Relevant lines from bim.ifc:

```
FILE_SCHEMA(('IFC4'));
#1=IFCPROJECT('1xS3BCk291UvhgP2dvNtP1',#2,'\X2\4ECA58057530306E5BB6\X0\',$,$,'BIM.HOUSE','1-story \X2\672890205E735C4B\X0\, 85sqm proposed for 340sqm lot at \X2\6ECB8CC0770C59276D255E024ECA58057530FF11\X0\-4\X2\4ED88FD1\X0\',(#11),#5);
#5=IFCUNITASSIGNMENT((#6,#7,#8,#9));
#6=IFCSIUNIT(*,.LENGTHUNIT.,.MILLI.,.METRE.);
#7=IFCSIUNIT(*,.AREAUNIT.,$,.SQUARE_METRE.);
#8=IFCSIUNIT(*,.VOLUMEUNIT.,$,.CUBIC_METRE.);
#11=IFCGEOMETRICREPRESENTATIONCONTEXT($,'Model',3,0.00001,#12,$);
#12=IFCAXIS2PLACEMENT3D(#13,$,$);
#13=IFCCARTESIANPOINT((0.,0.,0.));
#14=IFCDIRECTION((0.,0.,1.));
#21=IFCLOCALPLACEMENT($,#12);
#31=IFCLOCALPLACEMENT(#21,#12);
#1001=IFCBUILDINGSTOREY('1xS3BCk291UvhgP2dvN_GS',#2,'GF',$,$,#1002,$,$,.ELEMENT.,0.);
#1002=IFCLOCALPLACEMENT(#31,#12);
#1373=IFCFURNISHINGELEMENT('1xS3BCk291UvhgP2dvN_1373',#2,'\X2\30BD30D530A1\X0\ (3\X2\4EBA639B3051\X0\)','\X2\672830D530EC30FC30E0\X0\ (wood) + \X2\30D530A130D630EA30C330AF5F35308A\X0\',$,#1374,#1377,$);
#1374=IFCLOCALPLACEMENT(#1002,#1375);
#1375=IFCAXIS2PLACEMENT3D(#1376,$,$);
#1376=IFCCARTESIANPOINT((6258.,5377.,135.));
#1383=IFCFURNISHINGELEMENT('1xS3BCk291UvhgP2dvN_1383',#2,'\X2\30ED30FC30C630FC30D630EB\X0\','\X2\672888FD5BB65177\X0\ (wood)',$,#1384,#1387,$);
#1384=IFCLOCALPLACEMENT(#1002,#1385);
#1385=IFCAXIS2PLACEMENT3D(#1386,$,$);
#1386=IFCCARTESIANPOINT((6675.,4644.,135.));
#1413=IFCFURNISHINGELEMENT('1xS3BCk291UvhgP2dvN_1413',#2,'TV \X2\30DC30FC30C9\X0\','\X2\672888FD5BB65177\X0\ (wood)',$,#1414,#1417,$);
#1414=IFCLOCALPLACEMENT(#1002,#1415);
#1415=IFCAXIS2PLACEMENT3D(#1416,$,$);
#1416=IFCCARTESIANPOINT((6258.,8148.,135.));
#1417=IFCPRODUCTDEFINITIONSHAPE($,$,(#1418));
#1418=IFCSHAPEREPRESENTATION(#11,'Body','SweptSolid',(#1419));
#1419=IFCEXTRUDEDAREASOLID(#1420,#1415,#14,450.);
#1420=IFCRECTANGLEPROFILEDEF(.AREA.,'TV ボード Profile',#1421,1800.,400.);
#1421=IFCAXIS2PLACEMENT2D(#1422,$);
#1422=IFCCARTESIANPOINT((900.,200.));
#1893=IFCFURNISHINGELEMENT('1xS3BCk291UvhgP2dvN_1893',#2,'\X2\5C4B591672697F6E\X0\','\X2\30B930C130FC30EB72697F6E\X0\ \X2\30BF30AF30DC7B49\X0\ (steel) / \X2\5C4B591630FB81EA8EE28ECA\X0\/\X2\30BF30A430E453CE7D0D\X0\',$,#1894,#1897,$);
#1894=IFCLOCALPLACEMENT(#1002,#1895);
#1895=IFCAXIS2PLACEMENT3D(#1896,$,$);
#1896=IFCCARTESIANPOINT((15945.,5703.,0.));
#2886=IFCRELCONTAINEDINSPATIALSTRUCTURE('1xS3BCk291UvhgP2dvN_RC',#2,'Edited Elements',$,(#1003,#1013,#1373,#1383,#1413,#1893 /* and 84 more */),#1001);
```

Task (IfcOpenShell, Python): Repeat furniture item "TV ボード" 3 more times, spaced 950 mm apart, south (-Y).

```python
import numpy as np
import ifcopenshell
import ifcopenshell.api.geometry
import ifcopenshell.api.root
import ifcopenshell.util.element
import ifcopenshell.util.placement

model = ifcopenshell.open("bim.ifc")


def reuse_history(source, copy):
    """copy_class also copies each property set's owner history, people and application; keep the originals."""
    for rel in copy.IsDefinedBy:
        if rel.is_a("IfcRelDefinesByProperties") and (history := rel.RelatingPropertyDefinition.OwnerHistory):
            rel.RelatingPropertyDefinition.OwnerHistory = source.OwnerHistory
            ifcopenshell.util.element.remove_deep2(model, history)


source = model.by_id(1413)
base = ifcopenshell.util.placement.get_local_placement(source.ObjectPlacement)
step = np.array([0.0, -1.0, 0.0]) * 950.0

for i in range(1, 4):
    copy = ifcopenshell.api.root.copy_class(model, product=source)
    copy.Representation = ifcopenshell.util.element.copy_deep(
        model, source.Representation, exclude=["IfcGeometricRepresentationContext", "IfcRepresentationMap"]
    )
    reuse_history(source, copy)
    matrix = base.copy()
    matrix[:3, 3] += i * step
    print("added at", matrix[:3, 3].round(3) + 0.0)
    ifcopenshell.api.geometry.edit_object_placement(model, product=copy, matrix=matrix, is_si=False)

model.write("bim-out.ifc")
```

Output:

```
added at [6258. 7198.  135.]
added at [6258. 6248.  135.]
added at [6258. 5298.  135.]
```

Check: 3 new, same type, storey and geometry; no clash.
